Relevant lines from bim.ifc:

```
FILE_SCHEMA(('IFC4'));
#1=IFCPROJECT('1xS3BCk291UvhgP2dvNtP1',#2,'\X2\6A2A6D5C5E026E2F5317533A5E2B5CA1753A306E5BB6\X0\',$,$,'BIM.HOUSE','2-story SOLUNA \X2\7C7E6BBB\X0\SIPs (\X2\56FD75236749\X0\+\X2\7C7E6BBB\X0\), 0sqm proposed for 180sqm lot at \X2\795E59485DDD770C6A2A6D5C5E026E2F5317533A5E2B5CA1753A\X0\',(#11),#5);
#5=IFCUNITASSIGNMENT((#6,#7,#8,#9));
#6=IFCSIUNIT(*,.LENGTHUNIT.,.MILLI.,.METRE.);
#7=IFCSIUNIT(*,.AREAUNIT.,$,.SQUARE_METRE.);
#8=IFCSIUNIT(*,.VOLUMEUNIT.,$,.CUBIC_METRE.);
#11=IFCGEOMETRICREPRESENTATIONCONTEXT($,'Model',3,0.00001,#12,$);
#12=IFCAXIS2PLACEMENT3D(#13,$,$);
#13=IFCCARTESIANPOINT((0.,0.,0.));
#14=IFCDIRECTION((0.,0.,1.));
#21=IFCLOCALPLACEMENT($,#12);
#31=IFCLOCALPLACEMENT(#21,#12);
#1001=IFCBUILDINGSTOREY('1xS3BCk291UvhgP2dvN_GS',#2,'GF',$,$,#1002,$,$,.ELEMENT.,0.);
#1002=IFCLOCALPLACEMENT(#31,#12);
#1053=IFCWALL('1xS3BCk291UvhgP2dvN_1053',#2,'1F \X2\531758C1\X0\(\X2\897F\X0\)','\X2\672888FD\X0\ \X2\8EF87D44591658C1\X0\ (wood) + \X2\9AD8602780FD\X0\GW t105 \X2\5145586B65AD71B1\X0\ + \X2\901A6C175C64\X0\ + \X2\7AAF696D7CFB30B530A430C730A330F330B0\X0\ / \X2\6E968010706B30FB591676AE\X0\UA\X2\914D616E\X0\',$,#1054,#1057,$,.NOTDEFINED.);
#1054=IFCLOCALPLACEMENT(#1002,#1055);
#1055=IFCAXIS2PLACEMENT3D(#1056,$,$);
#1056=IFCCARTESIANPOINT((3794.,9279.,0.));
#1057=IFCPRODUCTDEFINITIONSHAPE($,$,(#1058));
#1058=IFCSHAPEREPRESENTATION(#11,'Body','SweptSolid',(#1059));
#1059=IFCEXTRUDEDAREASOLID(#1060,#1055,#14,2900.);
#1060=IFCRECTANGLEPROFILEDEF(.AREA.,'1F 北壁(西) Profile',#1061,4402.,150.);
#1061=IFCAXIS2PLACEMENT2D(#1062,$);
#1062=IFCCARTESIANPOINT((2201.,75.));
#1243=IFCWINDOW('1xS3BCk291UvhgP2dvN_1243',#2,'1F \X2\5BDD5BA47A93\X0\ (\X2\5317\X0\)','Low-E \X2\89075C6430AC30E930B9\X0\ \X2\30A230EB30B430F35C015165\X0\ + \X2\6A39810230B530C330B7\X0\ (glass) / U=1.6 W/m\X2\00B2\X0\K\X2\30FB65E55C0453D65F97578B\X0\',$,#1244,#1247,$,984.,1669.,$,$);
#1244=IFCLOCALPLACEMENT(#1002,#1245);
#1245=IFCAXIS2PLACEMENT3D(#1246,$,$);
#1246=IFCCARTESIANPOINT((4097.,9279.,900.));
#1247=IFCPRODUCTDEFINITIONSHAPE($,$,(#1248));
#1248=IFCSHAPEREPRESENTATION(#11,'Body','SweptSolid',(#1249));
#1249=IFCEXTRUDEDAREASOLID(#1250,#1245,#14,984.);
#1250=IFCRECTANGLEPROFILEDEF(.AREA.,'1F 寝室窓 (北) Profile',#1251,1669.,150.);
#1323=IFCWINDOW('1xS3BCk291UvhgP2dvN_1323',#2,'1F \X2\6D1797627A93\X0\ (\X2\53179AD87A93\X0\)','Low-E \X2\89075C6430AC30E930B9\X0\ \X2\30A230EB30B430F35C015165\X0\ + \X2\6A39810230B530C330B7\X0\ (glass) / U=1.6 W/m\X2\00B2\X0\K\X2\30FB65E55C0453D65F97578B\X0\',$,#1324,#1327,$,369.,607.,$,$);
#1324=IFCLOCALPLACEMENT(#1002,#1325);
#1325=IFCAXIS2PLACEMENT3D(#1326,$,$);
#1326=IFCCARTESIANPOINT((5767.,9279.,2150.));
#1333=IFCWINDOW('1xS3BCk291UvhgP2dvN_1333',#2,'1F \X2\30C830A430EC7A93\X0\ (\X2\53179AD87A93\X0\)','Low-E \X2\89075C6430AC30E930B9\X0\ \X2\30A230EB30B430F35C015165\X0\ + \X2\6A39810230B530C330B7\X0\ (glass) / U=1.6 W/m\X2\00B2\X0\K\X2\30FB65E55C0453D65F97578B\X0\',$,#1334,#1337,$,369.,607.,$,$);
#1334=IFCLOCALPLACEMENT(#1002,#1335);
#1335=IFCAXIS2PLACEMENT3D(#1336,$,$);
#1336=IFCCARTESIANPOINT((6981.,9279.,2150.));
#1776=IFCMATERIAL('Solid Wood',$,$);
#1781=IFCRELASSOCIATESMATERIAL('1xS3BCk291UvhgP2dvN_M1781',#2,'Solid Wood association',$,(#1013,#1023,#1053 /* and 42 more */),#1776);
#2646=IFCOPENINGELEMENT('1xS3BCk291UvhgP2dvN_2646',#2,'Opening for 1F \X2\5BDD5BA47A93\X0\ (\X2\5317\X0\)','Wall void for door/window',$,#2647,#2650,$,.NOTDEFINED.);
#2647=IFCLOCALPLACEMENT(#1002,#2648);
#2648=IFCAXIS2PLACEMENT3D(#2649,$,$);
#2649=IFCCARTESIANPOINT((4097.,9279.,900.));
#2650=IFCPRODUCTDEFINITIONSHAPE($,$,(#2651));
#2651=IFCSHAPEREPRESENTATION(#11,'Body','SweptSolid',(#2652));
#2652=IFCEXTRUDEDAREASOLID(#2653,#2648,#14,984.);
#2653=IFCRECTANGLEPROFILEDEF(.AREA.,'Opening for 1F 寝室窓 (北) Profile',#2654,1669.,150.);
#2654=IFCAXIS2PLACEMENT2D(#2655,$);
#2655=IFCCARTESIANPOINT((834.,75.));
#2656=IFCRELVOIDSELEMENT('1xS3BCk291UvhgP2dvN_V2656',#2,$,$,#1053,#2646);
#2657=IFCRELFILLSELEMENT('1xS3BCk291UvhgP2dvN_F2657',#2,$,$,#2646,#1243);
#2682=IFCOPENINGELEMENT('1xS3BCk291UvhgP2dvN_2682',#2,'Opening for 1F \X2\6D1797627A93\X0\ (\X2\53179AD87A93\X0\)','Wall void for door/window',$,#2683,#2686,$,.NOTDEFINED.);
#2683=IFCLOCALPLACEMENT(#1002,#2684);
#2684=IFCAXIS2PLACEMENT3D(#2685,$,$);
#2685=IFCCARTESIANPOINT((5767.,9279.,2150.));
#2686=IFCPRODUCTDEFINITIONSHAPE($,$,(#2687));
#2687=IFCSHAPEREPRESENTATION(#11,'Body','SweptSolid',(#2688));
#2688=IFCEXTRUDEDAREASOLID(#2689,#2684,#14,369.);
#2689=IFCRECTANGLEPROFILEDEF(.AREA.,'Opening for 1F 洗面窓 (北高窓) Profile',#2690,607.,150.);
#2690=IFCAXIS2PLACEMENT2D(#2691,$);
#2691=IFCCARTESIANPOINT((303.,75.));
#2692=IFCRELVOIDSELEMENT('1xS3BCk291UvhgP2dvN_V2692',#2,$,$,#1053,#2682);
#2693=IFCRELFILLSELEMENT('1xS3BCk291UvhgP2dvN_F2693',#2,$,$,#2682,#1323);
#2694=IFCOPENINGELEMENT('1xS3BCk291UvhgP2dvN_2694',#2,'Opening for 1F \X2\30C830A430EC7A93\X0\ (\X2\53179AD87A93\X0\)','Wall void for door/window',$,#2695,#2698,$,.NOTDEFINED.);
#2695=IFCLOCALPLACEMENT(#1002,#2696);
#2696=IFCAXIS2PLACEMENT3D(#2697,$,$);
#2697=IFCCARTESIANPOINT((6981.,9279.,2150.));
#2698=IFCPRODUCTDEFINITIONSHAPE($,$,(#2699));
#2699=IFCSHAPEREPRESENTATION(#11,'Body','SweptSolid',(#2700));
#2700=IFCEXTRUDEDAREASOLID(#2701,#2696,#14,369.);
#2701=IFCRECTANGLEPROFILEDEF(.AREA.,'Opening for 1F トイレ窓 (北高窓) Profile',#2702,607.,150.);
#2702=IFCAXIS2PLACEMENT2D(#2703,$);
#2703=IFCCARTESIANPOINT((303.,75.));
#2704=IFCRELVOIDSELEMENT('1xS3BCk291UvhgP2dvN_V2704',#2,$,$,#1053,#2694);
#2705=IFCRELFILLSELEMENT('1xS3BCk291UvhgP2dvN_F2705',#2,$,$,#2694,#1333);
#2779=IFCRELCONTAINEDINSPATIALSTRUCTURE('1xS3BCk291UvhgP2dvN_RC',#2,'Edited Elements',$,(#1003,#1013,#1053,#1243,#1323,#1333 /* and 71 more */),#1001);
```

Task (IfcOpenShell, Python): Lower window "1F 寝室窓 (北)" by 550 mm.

```python
import numpy as np
import ifcopenshell
import ifcopenshell.api.geometry
import ifcopenshell.util.placement
import ifcopenshell.util.unit

model = ifcopenshell.open("bim.ifc")
unit_scale = ifcopenshell.util.unit.calculate_unit_scale(model)

window = model.by_guid("1xS3BCk291UvhgP2dvN_1243")
opening = window.FillsVoids[0].RelatingOpeningElement
dz = -0.55 / unit_scale

shift = np.array([0.0, 0.0, dz])
# The window is not placed relative to its opening, so move both.
for product in (opening, window):
    matrix = ifcopenshell.util.placement.get_local_placement(product.ObjectPlacement)
    matrix[:3, 3] += shift
    ifcopenshell.api.geometry.edit_object_placement(model, product=product, matrix=matrix, is_si=False)

print(f"moved by {dz * unit_scale:+.3f} m")

model.write("bim-out.ifc")
```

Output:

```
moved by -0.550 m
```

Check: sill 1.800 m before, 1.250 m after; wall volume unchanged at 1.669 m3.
